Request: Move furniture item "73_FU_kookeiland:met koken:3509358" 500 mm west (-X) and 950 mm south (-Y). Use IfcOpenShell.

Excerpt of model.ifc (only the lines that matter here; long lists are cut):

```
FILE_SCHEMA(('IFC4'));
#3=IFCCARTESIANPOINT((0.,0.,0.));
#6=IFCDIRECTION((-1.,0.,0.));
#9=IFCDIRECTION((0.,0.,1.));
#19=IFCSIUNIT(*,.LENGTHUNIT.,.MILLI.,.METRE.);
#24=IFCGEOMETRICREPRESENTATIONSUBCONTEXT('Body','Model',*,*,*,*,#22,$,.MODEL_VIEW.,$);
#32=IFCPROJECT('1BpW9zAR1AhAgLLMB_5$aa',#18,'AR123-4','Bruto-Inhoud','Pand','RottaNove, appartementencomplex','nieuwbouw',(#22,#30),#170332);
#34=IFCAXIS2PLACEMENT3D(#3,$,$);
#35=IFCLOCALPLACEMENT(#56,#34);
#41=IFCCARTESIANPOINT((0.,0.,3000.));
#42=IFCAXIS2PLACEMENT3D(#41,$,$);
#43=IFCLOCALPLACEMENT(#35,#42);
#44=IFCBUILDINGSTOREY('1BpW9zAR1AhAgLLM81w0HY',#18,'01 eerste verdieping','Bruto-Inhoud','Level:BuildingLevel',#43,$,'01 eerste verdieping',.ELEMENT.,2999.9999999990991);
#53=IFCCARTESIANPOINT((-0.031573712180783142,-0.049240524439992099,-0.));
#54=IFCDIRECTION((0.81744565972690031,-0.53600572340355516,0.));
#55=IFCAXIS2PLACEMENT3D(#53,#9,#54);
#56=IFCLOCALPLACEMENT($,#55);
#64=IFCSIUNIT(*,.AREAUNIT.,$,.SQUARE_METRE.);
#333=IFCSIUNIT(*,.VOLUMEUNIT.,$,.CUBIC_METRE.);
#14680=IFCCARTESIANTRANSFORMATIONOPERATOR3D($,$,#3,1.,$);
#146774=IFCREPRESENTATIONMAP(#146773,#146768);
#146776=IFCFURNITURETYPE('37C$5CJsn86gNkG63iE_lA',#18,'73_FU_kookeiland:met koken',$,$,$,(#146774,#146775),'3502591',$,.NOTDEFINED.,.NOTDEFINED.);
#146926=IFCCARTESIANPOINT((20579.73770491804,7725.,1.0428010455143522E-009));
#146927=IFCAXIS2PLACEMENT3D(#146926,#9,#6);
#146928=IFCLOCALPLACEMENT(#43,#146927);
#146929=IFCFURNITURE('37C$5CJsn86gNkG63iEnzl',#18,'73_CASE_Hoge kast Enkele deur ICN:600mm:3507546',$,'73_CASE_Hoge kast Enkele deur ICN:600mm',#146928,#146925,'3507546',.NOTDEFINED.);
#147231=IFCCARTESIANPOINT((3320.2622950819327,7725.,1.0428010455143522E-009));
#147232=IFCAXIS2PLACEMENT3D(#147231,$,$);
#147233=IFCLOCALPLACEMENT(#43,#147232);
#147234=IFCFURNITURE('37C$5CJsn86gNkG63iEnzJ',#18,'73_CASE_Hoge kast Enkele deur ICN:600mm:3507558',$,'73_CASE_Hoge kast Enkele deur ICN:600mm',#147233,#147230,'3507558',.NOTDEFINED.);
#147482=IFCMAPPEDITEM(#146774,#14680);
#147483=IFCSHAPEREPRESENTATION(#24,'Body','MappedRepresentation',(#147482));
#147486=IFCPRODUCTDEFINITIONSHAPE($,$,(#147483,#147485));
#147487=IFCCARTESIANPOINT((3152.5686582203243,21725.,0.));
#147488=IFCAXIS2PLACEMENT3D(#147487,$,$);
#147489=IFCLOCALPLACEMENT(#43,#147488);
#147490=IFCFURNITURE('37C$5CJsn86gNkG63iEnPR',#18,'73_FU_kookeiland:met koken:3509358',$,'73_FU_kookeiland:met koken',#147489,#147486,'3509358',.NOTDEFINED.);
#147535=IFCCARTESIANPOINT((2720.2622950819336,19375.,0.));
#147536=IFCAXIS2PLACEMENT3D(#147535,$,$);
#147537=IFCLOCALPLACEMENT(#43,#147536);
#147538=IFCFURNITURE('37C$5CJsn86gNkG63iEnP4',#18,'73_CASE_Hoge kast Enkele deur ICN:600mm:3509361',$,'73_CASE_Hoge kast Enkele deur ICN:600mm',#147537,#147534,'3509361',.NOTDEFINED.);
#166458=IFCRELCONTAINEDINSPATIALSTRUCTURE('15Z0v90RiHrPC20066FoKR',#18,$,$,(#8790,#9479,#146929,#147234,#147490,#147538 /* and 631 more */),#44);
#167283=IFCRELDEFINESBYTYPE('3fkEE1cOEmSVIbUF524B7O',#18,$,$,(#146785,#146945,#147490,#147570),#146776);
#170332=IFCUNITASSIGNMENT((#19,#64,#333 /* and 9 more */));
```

```python
import ifcopenshell
import ifcopenshell.api.geometry
import ifcopenshell.util.placement
import ifcopenshell.util.unit

model = ifcopenshell.open("model.ifc")
unit_scale = ifcopenshell.util.unit.calculate_unit_scale(model)

item = model.by_guid("37C$5CJsn86gNkG63iEnPR")
matrix = ifcopenshell.util.placement.get_local_placement(item.ObjectPlacement)
matrix[0, 3] -= 0.5 / unit_scale
matrix[1, 3] -= 0.95 / unit_scale
ifcopenshell.api.geometry.edit_object_placement(model, product=item, matrix=matrix, is_si=False)

print(ifcopenshell.util.placement.get_local_placement(item.ObjectPlacement).round(3) + 0.0)

model.write("model_rev.ifc")
```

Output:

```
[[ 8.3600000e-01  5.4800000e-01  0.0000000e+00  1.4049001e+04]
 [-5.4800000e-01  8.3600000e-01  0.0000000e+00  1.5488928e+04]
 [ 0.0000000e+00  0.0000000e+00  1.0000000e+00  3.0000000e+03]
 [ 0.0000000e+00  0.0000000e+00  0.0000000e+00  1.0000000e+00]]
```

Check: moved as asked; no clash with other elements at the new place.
